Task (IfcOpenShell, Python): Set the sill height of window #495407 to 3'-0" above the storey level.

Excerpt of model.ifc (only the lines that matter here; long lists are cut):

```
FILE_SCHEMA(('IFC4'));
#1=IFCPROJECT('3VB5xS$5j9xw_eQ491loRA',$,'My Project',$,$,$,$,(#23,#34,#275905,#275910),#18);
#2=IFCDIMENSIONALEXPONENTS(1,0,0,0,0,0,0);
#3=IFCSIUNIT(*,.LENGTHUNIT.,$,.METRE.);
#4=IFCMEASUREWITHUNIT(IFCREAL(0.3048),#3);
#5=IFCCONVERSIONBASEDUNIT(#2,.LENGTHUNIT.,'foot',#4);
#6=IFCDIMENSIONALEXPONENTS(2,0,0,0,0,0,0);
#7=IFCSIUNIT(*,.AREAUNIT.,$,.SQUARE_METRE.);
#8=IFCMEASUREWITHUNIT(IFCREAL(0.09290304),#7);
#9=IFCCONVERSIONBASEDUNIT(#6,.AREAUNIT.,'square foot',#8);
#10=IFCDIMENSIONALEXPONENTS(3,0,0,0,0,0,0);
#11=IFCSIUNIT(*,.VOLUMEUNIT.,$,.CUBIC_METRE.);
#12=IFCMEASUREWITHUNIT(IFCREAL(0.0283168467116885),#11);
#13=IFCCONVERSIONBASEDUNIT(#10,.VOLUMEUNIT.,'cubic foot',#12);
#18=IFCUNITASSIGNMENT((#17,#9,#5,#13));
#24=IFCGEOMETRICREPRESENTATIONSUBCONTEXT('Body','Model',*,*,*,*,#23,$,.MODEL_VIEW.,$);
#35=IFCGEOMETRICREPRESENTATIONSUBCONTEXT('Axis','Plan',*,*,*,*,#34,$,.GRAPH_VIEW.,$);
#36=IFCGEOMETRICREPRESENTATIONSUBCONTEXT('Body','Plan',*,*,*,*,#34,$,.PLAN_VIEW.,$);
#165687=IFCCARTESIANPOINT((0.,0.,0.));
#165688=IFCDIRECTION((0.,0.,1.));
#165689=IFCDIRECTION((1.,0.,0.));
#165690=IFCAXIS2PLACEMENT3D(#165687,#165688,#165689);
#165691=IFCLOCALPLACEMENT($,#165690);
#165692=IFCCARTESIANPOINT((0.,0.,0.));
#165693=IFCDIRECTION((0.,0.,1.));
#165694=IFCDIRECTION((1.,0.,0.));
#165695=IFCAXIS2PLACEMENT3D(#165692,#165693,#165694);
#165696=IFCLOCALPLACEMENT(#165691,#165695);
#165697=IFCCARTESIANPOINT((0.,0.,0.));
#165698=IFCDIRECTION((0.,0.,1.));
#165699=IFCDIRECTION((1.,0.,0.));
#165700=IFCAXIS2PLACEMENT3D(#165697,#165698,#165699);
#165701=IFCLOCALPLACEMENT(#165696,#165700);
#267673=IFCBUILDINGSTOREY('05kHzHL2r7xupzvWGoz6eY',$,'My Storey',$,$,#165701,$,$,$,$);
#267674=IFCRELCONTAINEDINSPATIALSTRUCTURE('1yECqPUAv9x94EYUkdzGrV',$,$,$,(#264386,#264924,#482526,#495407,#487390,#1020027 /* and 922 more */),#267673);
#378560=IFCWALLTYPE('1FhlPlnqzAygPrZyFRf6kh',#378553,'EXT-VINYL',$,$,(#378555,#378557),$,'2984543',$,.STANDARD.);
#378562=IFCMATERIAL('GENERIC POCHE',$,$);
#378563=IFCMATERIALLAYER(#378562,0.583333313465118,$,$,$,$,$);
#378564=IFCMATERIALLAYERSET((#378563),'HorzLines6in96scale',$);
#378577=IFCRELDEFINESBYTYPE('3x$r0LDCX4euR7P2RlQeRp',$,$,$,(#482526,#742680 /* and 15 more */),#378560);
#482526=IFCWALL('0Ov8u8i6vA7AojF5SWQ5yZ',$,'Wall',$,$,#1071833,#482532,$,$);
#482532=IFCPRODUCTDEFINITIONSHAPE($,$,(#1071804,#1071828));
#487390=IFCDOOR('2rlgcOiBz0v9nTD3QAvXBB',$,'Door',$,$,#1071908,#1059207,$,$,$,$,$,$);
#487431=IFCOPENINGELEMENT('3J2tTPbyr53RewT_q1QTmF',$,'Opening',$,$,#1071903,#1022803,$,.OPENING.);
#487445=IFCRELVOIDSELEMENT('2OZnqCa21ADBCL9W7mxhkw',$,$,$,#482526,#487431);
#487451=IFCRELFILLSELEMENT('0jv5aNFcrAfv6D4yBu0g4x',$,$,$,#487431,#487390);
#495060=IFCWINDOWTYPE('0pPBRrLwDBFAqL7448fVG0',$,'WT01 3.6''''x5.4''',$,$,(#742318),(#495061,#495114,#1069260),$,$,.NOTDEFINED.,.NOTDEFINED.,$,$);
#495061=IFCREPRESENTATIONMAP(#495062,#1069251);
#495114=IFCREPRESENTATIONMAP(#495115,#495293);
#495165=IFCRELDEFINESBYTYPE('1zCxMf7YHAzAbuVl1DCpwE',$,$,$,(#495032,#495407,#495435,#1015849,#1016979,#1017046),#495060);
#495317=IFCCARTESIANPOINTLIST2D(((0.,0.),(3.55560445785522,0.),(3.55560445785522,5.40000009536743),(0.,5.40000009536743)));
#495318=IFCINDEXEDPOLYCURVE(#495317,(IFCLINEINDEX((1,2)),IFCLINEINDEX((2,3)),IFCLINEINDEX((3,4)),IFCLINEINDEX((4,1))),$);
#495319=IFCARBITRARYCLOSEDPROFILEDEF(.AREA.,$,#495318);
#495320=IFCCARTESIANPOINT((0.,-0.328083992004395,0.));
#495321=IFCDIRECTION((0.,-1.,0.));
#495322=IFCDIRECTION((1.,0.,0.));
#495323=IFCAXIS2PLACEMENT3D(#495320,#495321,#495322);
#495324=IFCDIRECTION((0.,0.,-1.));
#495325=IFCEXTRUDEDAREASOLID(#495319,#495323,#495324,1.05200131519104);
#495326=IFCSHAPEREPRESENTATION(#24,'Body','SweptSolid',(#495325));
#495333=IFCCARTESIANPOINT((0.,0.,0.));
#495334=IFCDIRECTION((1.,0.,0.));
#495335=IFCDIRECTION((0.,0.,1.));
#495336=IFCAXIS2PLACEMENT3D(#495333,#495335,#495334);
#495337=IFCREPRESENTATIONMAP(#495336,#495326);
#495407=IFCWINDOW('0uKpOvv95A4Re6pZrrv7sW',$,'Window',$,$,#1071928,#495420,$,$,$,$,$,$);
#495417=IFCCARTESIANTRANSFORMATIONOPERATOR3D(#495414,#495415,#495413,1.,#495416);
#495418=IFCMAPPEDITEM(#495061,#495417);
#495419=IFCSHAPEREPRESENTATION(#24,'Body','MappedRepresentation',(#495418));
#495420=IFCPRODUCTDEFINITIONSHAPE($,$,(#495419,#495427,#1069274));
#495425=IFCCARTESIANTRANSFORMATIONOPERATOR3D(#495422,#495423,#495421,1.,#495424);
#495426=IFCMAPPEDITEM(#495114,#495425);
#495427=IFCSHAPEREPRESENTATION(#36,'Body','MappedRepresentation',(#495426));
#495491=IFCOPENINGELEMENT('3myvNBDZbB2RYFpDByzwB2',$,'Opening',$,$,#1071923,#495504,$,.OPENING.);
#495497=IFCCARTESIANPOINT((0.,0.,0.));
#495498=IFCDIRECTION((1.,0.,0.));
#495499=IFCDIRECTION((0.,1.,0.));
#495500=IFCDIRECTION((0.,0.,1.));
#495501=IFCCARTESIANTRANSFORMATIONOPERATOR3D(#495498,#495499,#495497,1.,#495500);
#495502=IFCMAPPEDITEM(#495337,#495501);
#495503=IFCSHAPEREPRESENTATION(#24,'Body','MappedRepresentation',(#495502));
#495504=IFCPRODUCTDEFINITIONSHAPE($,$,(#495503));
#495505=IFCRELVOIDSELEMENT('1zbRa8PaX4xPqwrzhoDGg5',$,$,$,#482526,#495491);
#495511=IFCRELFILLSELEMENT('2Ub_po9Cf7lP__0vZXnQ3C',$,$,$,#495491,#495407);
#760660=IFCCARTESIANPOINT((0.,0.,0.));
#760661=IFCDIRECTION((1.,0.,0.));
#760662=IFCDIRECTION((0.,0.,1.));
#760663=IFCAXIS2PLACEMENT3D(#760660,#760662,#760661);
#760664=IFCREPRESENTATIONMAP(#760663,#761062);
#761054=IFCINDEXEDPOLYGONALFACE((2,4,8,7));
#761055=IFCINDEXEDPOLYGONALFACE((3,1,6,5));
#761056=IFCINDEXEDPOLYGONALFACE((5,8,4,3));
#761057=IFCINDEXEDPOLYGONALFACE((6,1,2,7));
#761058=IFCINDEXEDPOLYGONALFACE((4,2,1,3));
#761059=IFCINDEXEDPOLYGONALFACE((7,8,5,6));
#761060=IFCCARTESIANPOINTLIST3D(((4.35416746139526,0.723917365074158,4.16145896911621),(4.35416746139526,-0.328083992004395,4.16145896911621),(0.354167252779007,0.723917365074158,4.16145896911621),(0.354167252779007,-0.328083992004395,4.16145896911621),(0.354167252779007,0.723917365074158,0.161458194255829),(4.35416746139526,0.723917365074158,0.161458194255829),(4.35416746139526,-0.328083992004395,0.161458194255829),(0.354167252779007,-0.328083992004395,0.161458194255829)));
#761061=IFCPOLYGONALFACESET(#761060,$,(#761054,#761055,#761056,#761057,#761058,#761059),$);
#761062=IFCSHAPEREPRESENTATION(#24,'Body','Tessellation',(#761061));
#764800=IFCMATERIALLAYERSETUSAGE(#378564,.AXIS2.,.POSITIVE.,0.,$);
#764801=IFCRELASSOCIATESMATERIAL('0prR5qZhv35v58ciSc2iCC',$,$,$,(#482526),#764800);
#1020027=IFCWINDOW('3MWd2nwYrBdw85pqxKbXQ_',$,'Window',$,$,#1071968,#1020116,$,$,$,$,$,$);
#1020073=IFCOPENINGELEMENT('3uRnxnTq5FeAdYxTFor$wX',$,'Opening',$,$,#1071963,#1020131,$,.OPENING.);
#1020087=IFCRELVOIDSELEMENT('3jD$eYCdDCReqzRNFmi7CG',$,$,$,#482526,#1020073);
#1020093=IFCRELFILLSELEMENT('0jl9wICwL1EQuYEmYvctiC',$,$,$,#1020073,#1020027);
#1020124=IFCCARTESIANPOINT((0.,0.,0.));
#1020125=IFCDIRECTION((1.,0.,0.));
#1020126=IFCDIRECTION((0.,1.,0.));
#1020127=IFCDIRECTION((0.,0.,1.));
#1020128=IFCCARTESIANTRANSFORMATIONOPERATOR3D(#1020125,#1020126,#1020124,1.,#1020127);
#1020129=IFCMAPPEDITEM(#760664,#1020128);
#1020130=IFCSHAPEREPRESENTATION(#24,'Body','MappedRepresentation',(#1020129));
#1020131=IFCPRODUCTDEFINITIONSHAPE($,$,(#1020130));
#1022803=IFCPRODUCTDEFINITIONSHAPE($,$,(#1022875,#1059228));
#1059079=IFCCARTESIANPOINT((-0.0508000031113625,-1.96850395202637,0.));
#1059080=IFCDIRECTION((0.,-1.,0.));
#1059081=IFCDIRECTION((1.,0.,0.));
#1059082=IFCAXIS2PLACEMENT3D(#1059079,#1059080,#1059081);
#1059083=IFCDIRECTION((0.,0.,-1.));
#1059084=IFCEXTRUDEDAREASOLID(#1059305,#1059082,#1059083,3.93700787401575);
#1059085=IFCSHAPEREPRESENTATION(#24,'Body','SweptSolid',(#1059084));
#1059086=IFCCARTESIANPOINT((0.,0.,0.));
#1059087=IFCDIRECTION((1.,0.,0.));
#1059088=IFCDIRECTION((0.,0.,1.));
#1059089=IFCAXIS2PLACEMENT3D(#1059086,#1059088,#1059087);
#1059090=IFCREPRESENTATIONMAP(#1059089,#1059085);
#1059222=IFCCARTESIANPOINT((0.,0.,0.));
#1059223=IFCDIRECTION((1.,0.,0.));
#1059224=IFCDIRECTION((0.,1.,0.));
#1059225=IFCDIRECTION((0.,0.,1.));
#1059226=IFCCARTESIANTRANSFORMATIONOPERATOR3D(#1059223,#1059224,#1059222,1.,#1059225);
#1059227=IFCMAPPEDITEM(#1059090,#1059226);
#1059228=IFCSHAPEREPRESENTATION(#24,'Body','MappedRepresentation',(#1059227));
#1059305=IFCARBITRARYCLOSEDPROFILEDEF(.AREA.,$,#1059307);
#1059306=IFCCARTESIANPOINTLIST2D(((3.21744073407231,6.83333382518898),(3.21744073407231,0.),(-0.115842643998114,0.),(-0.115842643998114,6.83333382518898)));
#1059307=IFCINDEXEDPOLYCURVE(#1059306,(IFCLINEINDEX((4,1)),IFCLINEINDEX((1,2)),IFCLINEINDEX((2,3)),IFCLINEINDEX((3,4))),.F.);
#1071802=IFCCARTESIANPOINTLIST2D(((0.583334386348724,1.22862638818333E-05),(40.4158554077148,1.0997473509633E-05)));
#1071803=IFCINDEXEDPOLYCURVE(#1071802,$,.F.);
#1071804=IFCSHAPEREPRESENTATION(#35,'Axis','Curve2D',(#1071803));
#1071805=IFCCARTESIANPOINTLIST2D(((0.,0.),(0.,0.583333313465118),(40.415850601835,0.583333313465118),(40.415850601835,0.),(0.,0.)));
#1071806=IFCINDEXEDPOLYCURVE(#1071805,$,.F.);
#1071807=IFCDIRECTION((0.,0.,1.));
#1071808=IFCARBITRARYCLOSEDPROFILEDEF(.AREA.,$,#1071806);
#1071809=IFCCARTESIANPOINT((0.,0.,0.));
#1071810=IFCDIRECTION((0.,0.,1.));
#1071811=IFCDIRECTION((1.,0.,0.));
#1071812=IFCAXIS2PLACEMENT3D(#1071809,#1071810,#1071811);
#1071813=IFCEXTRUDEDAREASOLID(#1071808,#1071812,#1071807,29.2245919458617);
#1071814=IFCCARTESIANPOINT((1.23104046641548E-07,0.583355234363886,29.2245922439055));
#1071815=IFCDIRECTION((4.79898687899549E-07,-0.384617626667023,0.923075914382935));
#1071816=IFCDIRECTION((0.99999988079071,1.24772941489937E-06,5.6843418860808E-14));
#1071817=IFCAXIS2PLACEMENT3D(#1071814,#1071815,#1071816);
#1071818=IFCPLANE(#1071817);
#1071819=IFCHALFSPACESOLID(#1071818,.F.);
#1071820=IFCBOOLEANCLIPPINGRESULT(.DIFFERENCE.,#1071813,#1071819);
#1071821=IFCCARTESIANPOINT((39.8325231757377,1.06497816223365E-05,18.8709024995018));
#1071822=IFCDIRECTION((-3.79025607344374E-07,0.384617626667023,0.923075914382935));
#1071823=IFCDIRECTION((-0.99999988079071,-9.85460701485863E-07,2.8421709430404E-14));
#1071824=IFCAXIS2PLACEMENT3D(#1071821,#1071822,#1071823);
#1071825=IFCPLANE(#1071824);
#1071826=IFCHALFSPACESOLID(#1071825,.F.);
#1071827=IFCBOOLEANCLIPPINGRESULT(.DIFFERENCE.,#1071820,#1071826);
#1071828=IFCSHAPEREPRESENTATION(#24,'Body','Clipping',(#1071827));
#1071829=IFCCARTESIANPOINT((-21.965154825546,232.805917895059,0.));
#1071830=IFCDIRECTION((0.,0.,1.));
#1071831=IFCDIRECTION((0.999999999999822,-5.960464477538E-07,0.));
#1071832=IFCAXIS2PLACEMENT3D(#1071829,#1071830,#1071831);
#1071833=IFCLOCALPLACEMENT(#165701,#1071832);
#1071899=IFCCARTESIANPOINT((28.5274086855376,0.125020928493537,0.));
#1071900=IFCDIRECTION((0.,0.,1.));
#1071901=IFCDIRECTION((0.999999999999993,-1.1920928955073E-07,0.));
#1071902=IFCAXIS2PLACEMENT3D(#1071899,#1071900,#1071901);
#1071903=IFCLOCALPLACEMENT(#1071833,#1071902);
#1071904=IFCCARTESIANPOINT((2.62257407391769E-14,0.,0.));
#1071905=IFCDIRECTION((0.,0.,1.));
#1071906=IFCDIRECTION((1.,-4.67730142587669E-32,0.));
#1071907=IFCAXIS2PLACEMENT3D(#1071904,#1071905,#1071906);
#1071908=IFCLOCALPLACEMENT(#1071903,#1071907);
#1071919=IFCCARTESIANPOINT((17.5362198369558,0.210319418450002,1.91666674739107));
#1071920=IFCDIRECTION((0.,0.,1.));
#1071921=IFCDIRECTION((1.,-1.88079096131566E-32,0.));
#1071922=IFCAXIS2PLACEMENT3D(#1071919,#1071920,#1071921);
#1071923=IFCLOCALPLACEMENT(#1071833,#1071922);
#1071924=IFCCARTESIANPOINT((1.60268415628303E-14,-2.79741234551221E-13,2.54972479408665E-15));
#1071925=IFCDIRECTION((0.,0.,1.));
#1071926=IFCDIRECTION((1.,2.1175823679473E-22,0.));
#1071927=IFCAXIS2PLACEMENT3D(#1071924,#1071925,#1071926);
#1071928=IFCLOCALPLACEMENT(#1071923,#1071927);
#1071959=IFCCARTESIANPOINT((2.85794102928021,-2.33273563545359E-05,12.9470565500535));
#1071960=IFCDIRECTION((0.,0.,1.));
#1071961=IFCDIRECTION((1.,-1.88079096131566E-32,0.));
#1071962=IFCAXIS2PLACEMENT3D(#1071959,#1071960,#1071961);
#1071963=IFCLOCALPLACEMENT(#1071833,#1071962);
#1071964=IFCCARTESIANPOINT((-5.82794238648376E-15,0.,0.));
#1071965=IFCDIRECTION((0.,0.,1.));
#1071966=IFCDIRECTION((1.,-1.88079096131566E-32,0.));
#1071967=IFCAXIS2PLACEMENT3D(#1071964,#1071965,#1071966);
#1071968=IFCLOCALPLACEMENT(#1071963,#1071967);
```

```python
import numpy as np
import ifcopenshell
import ifcopenshell.api.geometry
import ifcopenshell.geom
import ifcopenshell.util.element
import ifcopenshell.util.placement
import ifcopenshell.util.shape
import ifcopenshell.util.unit

model = ifcopenshell.open("model.ifc")
unit_scale = ifcopenshell.util.unit.calculate_unit_scale(model)

window = model.by_id(495407)
opening = window.FillsVoids[0].RelatingOpeningElement
storey = ifcopenshell.util.element.get_container(window, ifc_class="IfcBuildingStorey")
level = ifcopenshell.util.placement.get_local_placement(storey.ObjectPlacement)[2, 3]

# The opening's origin need not be at the sill, so measure its lowest point.
shape = ifcopenshell.geom.create_shape(ifcopenshell.geom.settings(), opening)
bottom = ifcopenshell.util.shape.get_shape_bottom_elevation(shape, shape.geometry) / unit_scale
dz = level + 36 * 0.0254 / unit_scale - bottom

shift = np.array([0.0, 0.0, dz])
# The window is placed relative to its opening, so it follows when the opening moves.
matrix = ifcopenshell.util.placement.get_local_placement(opening.ObjectPlacement)
matrix[:3, 3] += shift
ifcopenshell.api.geometry.edit_object_placement(
    model, product=opening, matrix=matrix, is_si=False, should_transform_children=True
)

print(f"moved by {dz * unit_scale:+.3f} m")

model.write("model_edited.ifc")
```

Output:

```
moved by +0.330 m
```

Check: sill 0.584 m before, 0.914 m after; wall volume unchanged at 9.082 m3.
